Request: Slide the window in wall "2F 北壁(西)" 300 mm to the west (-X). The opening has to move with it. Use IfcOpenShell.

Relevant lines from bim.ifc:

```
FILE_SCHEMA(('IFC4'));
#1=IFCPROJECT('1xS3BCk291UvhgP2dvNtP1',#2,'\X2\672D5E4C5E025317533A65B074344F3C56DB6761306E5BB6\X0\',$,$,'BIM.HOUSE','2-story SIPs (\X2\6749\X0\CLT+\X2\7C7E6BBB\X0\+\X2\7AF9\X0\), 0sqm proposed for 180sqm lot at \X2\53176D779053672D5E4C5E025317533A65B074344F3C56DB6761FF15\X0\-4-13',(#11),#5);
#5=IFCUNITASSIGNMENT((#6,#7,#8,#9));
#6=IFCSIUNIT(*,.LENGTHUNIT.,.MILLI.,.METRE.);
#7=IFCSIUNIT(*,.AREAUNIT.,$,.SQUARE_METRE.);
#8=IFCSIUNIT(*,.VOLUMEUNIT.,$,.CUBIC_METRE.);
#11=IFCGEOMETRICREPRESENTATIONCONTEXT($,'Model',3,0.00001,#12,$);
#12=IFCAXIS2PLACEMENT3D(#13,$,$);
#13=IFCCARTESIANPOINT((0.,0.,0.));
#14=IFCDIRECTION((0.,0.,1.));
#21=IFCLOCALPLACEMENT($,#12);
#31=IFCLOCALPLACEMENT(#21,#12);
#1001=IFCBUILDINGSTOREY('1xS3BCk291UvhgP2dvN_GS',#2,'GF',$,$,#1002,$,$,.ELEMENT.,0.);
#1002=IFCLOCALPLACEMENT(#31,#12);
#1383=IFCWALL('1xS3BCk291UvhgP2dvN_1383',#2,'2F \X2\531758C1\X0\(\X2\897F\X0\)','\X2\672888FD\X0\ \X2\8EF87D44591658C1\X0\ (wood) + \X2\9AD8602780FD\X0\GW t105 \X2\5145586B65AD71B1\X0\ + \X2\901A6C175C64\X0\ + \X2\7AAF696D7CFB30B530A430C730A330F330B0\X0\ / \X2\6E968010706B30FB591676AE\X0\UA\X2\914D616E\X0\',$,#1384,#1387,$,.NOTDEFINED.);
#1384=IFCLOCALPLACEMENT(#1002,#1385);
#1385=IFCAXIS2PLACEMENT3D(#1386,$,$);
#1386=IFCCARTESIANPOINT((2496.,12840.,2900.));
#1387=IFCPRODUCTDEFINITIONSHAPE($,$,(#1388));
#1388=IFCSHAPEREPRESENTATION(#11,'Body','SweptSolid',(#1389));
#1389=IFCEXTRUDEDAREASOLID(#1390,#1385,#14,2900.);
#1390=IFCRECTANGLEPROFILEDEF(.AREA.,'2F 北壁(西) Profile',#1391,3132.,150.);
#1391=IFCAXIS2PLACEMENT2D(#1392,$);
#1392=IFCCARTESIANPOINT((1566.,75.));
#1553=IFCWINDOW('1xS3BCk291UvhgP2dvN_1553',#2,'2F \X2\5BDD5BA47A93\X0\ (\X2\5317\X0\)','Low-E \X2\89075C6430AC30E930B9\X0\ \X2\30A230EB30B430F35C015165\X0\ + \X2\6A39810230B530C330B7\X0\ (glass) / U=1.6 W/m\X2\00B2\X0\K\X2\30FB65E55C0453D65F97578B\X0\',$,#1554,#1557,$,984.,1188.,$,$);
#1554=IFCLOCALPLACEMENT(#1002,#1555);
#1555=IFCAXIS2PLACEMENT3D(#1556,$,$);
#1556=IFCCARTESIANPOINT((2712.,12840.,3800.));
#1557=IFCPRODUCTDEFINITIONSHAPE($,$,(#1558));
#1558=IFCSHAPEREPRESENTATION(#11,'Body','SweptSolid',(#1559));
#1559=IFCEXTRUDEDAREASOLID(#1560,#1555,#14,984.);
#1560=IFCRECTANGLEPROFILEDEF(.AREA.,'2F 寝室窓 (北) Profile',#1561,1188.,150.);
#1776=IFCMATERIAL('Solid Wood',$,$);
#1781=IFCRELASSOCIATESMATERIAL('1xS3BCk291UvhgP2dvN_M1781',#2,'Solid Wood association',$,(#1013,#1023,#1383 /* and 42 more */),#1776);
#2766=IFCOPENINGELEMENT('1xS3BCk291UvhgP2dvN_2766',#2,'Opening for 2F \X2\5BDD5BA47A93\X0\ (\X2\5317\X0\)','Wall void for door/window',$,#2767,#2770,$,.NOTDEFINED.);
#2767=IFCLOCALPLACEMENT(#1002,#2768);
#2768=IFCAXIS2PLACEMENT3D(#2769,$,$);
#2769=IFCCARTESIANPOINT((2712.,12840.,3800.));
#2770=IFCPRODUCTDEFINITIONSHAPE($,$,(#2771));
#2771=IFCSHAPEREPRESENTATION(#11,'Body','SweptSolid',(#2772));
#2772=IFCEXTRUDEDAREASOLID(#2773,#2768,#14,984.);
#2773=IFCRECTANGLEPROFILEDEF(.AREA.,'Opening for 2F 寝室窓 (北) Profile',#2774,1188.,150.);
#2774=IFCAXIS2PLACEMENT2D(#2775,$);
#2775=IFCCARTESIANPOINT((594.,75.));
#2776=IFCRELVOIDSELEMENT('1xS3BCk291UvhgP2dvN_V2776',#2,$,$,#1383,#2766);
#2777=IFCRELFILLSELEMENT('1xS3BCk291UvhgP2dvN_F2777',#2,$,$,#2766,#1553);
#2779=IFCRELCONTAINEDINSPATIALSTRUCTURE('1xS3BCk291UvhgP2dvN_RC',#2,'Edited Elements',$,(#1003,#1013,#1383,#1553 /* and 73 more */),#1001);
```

```python
import ifcopenshell
import ifcopenshell.api.geometry
import ifcopenshell.util.placement

model = ifcopenshell.open("bim.ifc")

window = model.by_guid("1xS3BCk291UvhgP2dvN_1553")
opening = window.FillsVoids[0].RelatingOpeningElement
wall = opening.VoidsElements[0].RelatingBuildingElement

wall_matrix = ifcopenshell.util.placement.get_local_placement(wall.ObjectPlacement)
shift = wall_matrix[:3, 0] * -300.0
before = ifcopenshell.util.placement.get_local_placement(window.ObjectPlacement)[:3, 3].copy()

# The window is not placed relative to its opening, so move both.
for product in (opening, window):
    matrix = ifcopenshell.util.placement.get_local_placement(product.ObjectPlacement)
    matrix[:3, 3] += shift
    ifcopenshell.api.geometry.edit_object_placement(model, product=product, matrix=matrix, is_si=False)

after = ifcopenshell.util.placement.get_local_placement(window.ObjectPlacement)[:3, 3]
print("window moved by", (after - before).round(3) + 0.0)

model.write("bim_v2.ifc")
```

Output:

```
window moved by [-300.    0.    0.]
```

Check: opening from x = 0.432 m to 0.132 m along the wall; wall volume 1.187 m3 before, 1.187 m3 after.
